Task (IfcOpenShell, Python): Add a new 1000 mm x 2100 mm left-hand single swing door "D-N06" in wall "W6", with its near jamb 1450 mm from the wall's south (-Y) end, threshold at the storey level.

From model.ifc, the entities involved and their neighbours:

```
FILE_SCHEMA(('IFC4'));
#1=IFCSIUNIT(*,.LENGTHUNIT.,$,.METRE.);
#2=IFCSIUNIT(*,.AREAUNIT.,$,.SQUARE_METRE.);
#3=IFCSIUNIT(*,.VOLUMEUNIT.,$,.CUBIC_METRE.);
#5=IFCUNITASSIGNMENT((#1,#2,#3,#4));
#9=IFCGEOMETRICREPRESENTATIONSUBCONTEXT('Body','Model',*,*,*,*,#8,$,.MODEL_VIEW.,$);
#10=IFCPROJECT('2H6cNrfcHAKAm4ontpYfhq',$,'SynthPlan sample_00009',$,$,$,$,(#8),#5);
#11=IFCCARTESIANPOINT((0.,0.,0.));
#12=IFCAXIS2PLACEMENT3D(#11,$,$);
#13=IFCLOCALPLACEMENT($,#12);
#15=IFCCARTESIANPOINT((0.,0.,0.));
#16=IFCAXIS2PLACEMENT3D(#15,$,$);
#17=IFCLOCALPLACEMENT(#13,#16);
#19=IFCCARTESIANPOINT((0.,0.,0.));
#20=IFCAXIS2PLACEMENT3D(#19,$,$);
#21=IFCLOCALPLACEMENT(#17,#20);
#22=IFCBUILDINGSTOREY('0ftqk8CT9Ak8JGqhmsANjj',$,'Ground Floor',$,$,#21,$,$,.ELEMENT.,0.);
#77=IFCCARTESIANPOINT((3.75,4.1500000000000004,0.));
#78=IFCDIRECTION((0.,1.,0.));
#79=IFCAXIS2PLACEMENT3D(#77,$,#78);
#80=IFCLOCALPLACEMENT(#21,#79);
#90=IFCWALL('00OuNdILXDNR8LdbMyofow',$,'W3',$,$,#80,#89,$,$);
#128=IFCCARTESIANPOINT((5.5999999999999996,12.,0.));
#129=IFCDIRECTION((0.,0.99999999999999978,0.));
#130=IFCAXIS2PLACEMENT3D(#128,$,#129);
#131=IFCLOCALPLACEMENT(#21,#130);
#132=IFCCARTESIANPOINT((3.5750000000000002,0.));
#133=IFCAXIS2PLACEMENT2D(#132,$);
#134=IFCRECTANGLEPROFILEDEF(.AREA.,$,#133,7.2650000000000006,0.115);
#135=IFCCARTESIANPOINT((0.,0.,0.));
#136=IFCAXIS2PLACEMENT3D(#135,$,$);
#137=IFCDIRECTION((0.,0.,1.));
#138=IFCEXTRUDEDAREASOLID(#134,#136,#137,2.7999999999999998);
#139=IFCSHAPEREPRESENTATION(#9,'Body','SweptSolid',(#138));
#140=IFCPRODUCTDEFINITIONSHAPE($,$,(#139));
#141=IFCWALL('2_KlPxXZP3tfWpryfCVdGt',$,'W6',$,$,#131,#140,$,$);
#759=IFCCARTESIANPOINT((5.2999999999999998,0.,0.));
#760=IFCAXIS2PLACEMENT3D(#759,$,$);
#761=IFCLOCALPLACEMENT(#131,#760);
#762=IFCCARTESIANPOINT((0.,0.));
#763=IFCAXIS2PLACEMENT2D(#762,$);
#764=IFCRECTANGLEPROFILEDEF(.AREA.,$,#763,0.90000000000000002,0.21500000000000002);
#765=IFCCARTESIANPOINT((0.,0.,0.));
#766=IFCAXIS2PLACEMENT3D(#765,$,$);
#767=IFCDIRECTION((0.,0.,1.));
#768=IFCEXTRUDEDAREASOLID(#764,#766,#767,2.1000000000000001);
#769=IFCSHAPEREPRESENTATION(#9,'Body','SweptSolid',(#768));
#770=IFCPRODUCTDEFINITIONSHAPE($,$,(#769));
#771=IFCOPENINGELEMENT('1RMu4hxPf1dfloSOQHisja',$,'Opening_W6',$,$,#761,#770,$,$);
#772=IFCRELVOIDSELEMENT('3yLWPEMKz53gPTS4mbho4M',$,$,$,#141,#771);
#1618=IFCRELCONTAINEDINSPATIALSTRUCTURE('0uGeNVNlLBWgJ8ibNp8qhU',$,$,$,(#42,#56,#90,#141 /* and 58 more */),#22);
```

```python
import numpy as np
import ifcopenshell
import ifcopenshell.api.feature
import ifcopenshell.api.geometry
import ifcopenshell.api.root
import ifcopenshell.api.spatial
import ifcopenshell.geom
import ifcopenshell.util.element
import ifcopenshell.util.placement
import ifcopenshell.util.representation
import ifcopenshell.util.shape
import ifcopenshell.util.unit

model = ifcopenshell.open("model.ifc")
unit_scale = ifcopenshell.util.unit.calculate_unit_scale(model)
settings = ifcopenshell.geom.settings()


def volume(element):
    """Net volume in cubic metres, openings subtracted."""
    shape = ifcopenshell.geom.create_shape(settings, element)
    return ifcopenshell.util.shape.get_volume(shape.geometry)


wall = model.by_guid("2_KlPxXZP3tfWpryfCVdGt")
storey = ifcopenshell.util.element.get_container(wall, ifc_class="IfcBuildingStorey")
context = ifcopenshell.util.representation.get_context(model, "Model", "Body", "MODEL_VIEW")
before = volume(wall)

width, height, from_end, sill = 1, 2.1, 1.45, 0.0  # metres

# The wall runs along its own X axis, and the end named is its -X end.
wall_shape = ifcopenshell.geom.create_shape(settings, wall)
x, y, z = ifcopenshell.util.shape.get_vertices(wall_shape.geometry).T
start = x.min() + from_end
face, thickness = float(y.min()), float(y.max() - y.min())
wall_matrix = ifcopenshell.util.placement.get_local_placement(wall.ObjectPlacement)
level = ifcopenshell.util.placement.get_local_placement(storey.ObjectPlacement)[2, 3]


def in_wall(x, y):
    """Placement at x, y metres in the wall's axes, at sill height."""
    matrix = wall_matrix.copy()
    matrix[:, 3] = wall_matrix @ np.array([x / unit_scale, y / unit_scale, 0.0, 1.0])
    matrix[2, 3] = level + sill / unit_scale
    return matrix


# Opening: a box that overshoots both wall faces by 50 mm.
opening = ifcopenshell.api.root.create_entity(model, ifc_class="IfcOpeningElement", predefined_type="OPENING")
box = ifcopenshell.api.geometry.add_wall_representation(
    model, context=context, length=width, height=height, thickness=thickness + 0.1
)
ifcopenshell.api.geometry.assign_representation(model, product=opening, representation=box)
ifcopenshell.api.geometry.edit_object_placement(model, product=opening, matrix=in_wall(start, face - 0.05), is_si=False)
ifcopenshell.api.feature.add_feature(model, feature=opening, element=wall)

door = ifcopenshell.api.root.create_entity(model, ifc_class="IfcDoor", name="D-N06", predefined_type="DOOR")
door.OverallWidth, door.OverallHeight = width / unit_scale, height / unit_scale
door.OperationType = "SINGLE_SWING_LEFT"
body = ifcopenshell.api.geometry.add_door_representation(
    model,
    context=context,
    overall_width=door.OverallWidth,
    overall_height=door.OverallHeight,
    operation_type="SINGLE_SWING_LEFT",
    lining_properties={"LiningDepth": thickness / unit_scale, "ThresholdDepth": thickness / unit_scale},
)
ifcopenshell.api.geometry.assign_representation(model, product=door, representation=body)
ifcopenshell.api.spatial.assign_container(model, products=[door], relating_structure=storey)
ifcopenshell.api.feature.add_filling(model, opening=opening, element=door)

# The lining spans the wall, so the door starts at the wall face.
ifcopenshell.api.geometry.edit_object_placement(model, product=door, matrix=in_wall(start, face), is_si=False)

after = volume(wall)

print(f"wall volume {before:.3f} -> {after:.3f} m3")

model.write("model_v2.ifc")
```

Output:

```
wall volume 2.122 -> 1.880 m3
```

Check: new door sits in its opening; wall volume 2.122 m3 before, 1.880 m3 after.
